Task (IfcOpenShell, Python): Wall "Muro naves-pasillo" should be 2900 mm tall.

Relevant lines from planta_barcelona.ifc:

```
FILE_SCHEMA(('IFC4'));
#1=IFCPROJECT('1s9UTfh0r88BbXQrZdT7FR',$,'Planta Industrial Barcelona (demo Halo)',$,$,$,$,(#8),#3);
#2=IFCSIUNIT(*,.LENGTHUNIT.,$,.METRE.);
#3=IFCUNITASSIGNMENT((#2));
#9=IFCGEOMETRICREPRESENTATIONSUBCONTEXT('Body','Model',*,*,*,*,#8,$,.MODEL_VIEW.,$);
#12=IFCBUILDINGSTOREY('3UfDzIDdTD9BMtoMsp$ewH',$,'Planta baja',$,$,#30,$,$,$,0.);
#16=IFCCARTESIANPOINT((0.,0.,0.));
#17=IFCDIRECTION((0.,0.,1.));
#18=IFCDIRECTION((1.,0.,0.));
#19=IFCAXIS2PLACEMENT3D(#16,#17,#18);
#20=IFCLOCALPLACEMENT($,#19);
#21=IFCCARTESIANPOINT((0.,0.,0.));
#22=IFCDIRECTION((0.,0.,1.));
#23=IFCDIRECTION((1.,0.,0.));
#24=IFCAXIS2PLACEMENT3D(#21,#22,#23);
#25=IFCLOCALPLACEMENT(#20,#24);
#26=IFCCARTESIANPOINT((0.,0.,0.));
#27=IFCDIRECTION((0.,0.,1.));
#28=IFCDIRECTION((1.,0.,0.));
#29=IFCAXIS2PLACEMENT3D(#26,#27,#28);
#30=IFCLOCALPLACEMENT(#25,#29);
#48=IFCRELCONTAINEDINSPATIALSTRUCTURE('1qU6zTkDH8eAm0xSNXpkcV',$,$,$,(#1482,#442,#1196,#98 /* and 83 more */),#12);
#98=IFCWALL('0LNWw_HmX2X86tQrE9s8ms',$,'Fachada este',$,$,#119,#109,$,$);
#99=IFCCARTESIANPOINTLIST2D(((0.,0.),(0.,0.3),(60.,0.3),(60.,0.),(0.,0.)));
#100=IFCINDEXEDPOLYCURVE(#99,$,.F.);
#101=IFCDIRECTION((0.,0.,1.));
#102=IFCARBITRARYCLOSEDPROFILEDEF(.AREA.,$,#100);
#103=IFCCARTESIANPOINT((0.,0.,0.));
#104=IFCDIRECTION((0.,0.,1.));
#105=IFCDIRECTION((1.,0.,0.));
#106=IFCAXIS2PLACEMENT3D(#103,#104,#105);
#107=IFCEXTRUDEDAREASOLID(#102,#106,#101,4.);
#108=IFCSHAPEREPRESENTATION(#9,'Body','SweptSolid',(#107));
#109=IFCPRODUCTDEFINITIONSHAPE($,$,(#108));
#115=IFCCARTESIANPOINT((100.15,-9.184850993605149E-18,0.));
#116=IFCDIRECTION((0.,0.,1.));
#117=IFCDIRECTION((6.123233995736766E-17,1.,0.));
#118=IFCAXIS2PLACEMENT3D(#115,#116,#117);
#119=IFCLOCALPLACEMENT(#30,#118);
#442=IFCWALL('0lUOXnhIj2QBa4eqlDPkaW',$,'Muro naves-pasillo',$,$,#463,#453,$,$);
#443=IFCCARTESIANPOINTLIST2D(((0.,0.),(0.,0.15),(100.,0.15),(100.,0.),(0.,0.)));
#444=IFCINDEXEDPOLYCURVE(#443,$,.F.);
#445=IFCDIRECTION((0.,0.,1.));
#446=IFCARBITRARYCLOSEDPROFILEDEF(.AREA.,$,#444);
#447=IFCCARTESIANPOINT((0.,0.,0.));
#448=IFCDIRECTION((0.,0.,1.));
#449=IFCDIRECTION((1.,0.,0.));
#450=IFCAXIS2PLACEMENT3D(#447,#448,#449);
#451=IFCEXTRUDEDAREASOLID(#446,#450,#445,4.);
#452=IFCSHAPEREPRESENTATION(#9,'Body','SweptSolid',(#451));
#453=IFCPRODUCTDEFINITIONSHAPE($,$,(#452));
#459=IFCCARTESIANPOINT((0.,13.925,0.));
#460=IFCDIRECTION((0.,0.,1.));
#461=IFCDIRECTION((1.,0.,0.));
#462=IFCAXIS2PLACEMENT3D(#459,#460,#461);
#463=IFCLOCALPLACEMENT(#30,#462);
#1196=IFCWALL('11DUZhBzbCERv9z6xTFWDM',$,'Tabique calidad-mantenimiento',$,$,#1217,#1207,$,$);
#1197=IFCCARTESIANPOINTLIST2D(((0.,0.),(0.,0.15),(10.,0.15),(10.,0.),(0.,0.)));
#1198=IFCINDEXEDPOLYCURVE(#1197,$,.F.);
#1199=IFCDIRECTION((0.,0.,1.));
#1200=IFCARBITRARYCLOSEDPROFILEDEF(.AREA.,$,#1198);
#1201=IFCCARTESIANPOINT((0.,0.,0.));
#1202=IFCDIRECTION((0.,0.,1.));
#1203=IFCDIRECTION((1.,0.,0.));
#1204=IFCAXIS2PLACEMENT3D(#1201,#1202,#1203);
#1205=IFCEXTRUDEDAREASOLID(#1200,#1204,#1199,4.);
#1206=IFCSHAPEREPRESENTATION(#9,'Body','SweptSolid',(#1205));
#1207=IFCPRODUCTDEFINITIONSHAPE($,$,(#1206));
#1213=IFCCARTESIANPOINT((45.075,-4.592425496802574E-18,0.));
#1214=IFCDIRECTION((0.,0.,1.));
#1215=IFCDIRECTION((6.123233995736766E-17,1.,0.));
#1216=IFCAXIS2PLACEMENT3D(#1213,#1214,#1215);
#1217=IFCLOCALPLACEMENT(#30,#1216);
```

```python
import ifcopenshell
import ifcopenshell.geom
import ifcopenshell.util.representation
import ifcopenshell.util.shape
import ifcopenshell.util.unit

model = ifcopenshell.open("planta_barcelona.ifc")
unit_scale = ifcopenshell.util.unit.calculate_unit_scale(model)
settings = ifcopenshell.geom.settings()


def volume(element):
    """Net volume in cubic metres, openings subtracted."""
    shape = ifcopenshell.geom.create_shape(settings, element)
    return ifcopenshell.util.shape.get_volume(shape.geometry)


wall = model.by_guid("0lUOXnhIj2QBa4eqlDPkaW")
before = volume(wall)

body = ifcopenshell.util.representation.get_representation(wall, "Model", "Body")
solid = body.Items[0]
old_height = solid.Depth
solid.Depth = 2.9 / unit_scale
after = volume(wall)

print(f"height {old_height:g} -> {solid.Depth:g}, volume {before:.3f} -> {after:.3f} m3")

model.write("planta_barcelona_v2.ifc")
```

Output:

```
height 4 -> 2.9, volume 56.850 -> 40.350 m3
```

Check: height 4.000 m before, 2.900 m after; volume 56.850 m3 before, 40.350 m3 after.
